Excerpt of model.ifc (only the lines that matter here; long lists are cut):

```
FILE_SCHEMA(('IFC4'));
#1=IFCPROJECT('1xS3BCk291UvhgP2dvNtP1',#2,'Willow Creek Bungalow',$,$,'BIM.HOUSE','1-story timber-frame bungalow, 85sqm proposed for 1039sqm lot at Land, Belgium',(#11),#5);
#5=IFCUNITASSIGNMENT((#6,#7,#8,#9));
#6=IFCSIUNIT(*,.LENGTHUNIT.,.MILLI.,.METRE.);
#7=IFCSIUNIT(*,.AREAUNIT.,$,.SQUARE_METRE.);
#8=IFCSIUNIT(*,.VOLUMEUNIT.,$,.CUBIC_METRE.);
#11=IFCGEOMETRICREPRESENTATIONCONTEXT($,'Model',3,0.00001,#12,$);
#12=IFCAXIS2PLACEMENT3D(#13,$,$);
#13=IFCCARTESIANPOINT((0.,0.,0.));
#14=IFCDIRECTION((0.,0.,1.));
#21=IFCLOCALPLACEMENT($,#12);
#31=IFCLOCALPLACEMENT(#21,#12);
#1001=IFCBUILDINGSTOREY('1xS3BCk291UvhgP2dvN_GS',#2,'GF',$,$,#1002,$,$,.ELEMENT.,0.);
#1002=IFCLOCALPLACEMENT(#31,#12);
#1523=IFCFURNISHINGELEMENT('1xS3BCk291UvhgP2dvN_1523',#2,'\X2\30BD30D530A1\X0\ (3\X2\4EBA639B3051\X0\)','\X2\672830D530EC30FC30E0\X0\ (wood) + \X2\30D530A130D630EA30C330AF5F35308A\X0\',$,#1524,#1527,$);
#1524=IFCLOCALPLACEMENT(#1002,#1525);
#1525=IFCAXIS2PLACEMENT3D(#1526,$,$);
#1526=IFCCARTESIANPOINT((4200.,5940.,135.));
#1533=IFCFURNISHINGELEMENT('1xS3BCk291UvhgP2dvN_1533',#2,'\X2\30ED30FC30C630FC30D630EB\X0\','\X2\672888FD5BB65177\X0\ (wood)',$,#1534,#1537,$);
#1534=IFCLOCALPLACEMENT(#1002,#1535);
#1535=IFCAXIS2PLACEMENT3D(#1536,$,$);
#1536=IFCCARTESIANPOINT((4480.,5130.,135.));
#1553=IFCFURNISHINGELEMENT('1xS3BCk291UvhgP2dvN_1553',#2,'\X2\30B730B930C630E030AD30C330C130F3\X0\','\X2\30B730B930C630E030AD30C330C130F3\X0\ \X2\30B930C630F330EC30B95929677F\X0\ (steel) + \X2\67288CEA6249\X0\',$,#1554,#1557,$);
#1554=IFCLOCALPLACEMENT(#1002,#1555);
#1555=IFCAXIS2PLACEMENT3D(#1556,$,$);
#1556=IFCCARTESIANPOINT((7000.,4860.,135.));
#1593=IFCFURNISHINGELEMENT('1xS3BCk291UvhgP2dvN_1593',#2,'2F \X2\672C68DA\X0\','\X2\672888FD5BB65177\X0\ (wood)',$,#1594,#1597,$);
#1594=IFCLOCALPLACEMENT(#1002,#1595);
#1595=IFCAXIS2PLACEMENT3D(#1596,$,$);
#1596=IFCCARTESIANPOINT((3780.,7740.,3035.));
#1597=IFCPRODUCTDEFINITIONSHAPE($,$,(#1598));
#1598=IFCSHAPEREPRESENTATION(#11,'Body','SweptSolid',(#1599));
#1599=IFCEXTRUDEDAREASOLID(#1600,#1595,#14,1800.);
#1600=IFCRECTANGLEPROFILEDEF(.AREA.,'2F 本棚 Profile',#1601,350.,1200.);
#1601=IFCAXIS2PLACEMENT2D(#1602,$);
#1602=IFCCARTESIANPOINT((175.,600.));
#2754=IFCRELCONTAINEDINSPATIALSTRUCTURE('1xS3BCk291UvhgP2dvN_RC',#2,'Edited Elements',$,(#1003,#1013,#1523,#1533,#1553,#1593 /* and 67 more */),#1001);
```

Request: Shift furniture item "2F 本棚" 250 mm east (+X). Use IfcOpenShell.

```python
import ifcopenshell
import ifcopenshell.api.geometry
import ifcopenshell.util.placement
import ifcopenshell.util.unit

model = ifcopenshell.open("model.ifc")
unit_scale = ifcopenshell.util.unit.calculate_unit_scale(model)

item = model.by_id(1593)
matrix = ifcopenshell.util.placement.get_local_placement(item.ObjectPlacement)
matrix[0, 3] += 0.25 / unit_scale
ifcopenshell.api.geometry.edit_object_placement(model, product=item, matrix=matrix, is_si=False)

print(ifcopenshell.util.placement.get_local_placement(item.ObjectPlacement).round(3) + 0.0)

model.write("model_v2.ifc")
```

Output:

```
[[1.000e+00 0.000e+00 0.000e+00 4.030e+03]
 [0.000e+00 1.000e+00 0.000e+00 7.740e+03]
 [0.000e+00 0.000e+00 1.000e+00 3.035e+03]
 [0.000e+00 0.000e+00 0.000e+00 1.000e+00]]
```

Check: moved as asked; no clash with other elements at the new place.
